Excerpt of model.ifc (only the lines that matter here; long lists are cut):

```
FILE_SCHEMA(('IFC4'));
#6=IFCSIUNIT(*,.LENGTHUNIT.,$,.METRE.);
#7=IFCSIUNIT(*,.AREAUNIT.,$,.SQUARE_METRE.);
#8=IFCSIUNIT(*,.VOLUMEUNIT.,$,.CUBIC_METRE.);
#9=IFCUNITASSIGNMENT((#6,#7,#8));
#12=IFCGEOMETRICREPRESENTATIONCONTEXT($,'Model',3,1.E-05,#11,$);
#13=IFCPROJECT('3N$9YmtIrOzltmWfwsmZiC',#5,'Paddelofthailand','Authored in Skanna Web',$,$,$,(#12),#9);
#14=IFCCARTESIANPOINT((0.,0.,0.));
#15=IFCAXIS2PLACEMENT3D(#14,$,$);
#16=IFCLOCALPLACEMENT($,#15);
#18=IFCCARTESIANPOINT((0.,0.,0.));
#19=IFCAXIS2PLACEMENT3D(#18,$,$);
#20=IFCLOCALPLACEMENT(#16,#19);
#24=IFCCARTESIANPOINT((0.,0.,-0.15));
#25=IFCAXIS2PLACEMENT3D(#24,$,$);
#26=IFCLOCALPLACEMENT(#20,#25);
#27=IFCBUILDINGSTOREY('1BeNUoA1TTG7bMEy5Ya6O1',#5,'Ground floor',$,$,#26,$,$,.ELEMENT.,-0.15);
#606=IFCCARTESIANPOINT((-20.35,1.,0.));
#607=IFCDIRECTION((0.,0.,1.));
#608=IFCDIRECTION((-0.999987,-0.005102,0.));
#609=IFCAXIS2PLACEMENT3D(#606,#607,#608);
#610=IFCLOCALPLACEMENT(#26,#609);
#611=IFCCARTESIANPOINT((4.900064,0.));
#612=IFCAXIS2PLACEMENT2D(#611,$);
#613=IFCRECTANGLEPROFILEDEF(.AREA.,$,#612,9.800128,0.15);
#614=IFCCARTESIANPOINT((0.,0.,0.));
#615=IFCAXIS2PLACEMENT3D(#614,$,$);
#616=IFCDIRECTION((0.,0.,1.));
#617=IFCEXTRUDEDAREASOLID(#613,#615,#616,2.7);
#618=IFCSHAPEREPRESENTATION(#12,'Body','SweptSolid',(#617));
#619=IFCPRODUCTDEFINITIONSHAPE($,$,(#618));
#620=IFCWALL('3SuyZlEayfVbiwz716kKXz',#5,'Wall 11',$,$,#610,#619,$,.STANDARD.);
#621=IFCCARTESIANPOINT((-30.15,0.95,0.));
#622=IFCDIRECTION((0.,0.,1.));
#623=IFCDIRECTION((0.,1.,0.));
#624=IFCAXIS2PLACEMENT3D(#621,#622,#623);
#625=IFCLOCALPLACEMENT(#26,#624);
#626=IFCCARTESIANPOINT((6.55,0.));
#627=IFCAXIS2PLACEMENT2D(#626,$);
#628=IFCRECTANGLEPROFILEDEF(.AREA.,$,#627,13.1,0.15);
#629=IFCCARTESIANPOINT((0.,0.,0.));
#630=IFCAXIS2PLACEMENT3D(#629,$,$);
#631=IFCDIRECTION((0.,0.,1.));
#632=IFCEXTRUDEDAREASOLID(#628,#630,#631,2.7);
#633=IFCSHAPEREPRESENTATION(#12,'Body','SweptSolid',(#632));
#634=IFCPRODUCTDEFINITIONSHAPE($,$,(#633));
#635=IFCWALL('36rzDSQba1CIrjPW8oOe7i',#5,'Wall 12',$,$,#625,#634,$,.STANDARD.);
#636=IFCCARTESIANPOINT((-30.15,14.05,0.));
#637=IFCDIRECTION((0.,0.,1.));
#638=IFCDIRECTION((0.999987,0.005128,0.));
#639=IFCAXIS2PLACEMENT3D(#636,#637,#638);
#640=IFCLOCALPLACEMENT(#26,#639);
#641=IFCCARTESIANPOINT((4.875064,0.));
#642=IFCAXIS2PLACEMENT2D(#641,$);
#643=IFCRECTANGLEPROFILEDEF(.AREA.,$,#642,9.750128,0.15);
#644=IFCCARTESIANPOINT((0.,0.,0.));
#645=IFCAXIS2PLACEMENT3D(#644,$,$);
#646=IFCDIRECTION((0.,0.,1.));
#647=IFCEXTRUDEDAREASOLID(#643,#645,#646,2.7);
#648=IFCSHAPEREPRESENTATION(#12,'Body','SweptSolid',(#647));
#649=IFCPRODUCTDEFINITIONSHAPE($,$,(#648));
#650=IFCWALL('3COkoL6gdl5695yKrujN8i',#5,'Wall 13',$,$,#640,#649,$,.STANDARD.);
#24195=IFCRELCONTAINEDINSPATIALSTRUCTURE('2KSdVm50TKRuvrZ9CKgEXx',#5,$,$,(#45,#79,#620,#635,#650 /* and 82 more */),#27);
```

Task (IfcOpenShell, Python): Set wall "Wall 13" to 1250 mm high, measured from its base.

```python
import ifcopenshell
import ifcopenshell.geom
import ifcopenshell.util.shape

model = ifcopenshell.open("model.ifc")
settings = ifcopenshell.geom.settings()


def volume(element):
    """Net volume in cubic metres, openings subtracted."""
    shape = ifcopenshell.geom.create_shape(settings, element)
    return ifcopenshell.util.shape.get_volume(shape.geometry)


wall = model.by_guid("3COkoL6gdl5695yKrujN8i")
before = volume(wall)

body = next(r for r in wall.Representation.Representations if r.RepresentationIdentifier == "Body")
solid = body.Items[0]
old_height = solid.Depth
solid.Depth = 1.25
after = volume(wall)

print(f"height {old_height:g} -> {solid.Depth:g}, volume {before:.3f} -> {after:.3f} m3")

model.write("model_edited.ifc")
```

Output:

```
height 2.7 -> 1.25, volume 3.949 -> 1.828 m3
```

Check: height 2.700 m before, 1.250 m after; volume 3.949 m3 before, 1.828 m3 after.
